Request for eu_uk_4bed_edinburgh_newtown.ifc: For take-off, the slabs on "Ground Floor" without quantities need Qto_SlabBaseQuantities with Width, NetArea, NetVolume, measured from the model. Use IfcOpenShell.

First a look at what the model holds.

```python
import ifcopenshell
import ifcopenshell.util.element
import ifcopenshell.util.unit

model = ifcopenshell.open("eu_uk_4bed_edinburgh_newtown.ifc")
print(model.schema)
for unit_type in ("LENGTHUNIT", "AREAUNIT", "VOLUMEUNIT"):
    print(unit_type, ifcopenshell.util.unit.calculate_unit_scale(model, unit_type))
storey = next(s for s in model.by_type("IfcBuildingStorey") if s.Name == "Ground Floor")
slabs = [e for e in ifcopenshell.util.element.get_decomposition(storey) if e.is_a("IfcSlab")]
for e in sorted(slabs, key=lambda e: e.id()):
    print(e.id(), e.is_a(), e.Name, list(ifcopenshell.util.element.get_psets(e, qtos_only=True)), sep=" | ")
```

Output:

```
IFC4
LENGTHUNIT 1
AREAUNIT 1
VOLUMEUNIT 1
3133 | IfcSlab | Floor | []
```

```python
import ifcopenshell
import ifcopenshell.api.pset
import ifcopenshell.geom
import ifcopenshell.util.element
import ifcopenshell.util.shape
import ifcopenshell.util.unit

model = ifcopenshell.open("eu_uk_4bed_edinburgh_newtown.ifc")
unit_scale = ifcopenshell.util.unit.calculate_unit_scale(model)
area_scale = ifcopenshell.util.unit.calculate_unit_scale(model, "AREAUNIT")
volume_scale = ifcopenshell.util.unit.calculate_unit_scale(model, "VOLUMEUNIT")
settings = ifcopenshell.geom.settings()

storey = next(s for s in model.by_type("IfcBuildingStorey") if s.Name == "Ground Floor")
slabs = [e for e in ifcopenshell.util.element.get_decomposition(storey) if e.is_a("IfcSlab")]

for e in sorted(slabs, key=lambda e: e.id()):
    if ifcopenshell.util.element.get_psets(e, qtos_only=True, should_inherit=False):
        continue
    # Geometry comes back in metres, in the element's own axes.
    shape = ifcopenshell.geom.create_shape(settings, e)
    values = {
        "Width": ifcopenshell.util.shape.get_z(shape.geometry) / unit_scale,
        "NetArea": ifcopenshell.util.shape.get_footprint_area(shape.geometry) / area_scale,
        "NetVolume": ifcopenshell.util.shape.get_volume(shape.geometry) / volume_scale,
    }
    qto = ifcopenshell.api.pset.add_qto(model, product=e, name="Qto_SlabBaseQuantities")
    ifcopenshell.api.pset.edit_qto(model, qto=qto, properties=values)
    print(e.id(), {k: round(v, 3) for k, v in values.items()})

model.write("eu_uk_4bed_edinburgh_newtown_v2.ifc")
```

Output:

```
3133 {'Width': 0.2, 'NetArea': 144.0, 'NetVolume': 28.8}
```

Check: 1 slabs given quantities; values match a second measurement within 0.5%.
